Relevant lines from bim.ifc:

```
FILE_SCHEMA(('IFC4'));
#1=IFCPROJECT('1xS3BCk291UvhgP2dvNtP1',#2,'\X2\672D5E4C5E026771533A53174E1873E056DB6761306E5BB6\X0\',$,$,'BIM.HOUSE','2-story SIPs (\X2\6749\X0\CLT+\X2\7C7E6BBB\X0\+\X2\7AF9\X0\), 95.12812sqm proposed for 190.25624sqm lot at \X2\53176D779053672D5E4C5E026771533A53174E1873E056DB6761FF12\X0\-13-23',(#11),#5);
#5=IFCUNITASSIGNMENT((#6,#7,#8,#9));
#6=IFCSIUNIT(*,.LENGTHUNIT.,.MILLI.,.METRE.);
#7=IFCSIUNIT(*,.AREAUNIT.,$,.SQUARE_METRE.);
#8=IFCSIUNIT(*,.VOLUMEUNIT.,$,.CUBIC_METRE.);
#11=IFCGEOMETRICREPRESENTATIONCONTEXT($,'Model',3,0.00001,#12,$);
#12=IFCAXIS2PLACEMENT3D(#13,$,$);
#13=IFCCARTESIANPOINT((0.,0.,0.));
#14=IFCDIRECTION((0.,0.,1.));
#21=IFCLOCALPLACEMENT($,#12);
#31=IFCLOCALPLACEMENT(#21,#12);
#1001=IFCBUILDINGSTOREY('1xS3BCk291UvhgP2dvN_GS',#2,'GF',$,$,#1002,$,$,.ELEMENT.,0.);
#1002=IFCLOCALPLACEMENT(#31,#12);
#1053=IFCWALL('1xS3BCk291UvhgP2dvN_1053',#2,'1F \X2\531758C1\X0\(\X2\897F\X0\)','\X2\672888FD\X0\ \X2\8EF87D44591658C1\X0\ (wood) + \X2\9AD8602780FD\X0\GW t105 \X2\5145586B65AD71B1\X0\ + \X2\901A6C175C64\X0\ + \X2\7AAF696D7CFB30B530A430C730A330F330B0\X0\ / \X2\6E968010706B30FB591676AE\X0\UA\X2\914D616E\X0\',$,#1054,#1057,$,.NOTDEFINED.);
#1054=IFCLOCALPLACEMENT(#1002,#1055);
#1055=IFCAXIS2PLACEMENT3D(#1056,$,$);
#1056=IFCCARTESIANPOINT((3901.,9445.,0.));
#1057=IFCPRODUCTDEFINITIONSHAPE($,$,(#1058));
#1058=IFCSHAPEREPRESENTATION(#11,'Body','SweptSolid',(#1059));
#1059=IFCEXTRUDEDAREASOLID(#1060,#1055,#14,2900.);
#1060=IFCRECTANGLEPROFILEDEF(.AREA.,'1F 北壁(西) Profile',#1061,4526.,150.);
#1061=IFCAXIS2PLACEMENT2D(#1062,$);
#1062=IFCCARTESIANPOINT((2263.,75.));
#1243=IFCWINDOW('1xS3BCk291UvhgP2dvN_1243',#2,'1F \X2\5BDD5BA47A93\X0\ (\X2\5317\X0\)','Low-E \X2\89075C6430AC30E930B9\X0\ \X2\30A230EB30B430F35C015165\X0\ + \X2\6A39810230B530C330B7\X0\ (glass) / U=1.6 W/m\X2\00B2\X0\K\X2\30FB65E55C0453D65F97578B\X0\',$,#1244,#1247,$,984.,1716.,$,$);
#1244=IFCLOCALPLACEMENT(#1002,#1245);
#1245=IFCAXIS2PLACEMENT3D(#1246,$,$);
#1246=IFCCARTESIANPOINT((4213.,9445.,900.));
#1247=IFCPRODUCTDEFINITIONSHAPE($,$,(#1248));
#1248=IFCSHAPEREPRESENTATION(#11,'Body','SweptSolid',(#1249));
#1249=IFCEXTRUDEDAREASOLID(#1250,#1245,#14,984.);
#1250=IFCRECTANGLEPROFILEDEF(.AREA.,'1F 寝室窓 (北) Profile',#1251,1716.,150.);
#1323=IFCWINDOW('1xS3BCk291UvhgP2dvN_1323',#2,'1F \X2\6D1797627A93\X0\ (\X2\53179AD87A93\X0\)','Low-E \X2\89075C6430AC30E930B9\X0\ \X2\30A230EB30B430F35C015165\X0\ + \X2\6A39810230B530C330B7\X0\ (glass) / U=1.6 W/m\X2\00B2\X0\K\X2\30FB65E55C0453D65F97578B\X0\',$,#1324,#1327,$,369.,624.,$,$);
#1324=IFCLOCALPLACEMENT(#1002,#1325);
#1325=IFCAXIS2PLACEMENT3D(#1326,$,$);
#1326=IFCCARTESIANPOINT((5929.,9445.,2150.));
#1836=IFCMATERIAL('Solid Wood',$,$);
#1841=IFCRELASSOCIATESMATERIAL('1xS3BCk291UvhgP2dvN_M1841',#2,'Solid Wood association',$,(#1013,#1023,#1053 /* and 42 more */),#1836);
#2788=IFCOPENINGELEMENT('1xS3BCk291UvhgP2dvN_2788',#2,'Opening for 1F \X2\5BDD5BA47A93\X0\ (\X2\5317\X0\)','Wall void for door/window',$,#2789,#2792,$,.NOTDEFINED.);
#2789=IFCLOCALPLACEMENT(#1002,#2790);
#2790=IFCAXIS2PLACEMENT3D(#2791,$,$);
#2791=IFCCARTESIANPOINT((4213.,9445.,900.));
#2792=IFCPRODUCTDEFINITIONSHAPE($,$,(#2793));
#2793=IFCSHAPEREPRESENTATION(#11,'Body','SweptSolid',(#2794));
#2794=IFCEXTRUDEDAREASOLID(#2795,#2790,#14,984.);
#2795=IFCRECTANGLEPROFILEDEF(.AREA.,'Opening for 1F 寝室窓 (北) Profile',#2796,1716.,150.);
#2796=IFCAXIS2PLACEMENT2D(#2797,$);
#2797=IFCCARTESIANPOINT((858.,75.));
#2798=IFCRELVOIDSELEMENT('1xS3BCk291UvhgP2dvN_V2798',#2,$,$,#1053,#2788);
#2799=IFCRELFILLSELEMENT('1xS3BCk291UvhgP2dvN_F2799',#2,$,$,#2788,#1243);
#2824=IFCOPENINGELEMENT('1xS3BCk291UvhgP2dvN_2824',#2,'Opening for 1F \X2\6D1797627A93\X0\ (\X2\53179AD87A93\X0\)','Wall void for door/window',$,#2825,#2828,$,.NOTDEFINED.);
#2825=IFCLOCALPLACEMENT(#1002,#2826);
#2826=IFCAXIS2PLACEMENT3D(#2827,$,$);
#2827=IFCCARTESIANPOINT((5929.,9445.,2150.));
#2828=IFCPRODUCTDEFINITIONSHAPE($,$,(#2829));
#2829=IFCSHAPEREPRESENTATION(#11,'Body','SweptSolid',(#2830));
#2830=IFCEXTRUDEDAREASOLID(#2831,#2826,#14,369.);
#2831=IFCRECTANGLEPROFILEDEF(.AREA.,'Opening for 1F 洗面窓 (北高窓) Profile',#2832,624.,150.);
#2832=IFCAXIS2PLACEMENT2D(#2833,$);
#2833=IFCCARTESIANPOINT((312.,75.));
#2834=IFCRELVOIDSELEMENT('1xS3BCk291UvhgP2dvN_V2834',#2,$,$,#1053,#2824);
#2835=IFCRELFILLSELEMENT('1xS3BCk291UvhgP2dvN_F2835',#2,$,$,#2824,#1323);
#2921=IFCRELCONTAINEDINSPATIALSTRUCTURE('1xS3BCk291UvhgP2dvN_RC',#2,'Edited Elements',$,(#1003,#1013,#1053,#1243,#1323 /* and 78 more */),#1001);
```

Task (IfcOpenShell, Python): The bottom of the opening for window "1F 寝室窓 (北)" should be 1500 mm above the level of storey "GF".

```python
import numpy as np
import ifcopenshell
import ifcopenshell.api.geometry
import ifcopenshell.geom
import ifcopenshell.util.element
import ifcopenshell.util.placement
import ifcopenshell.util.shape
import ifcopenshell.util.unit

model = ifcopenshell.open("bim.ifc")
unit_scale = ifcopenshell.util.unit.calculate_unit_scale(model)

window = model.by_id(1243)
opening = window.FillsVoids[0].RelatingOpeningElement
storey = ifcopenshell.util.element.get_container(window, ifc_class="IfcBuildingStorey")
level = ifcopenshell.util.placement.get_local_placement(storey.ObjectPlacement)[2, 3]

# The opening's origin need not be at the sill, so measure its lowest point.
shape = ifcopenshell.geom.create_shape(ifcopenshell.geom.settings(), opening)
bottom = ifcopenshell.util.shape.get_shape_bottom_elevation(shape, shape.geometry) / unit_scale
dz = level + 1.5 / unit_scale - bottom

shift = np.array([0.0, 0.0, dz])
# The window is not placed relative to its opening, so move both.
for product in (opening, window):
    matrix = ifcopenshell.util.placement.get_local_placement(product.ObjectPlacement)
    matrix[:3, 3] += shift
    ifcopenshell.api.geometry.edit_object_placement(model, product=product, matrix=matrix, is_si=False)

print(f"moved by {dz * unit_scale:+.3f} m")

model.write("bim_updated.ifc")
```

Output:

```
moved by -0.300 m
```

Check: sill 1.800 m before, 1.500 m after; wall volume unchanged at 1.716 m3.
